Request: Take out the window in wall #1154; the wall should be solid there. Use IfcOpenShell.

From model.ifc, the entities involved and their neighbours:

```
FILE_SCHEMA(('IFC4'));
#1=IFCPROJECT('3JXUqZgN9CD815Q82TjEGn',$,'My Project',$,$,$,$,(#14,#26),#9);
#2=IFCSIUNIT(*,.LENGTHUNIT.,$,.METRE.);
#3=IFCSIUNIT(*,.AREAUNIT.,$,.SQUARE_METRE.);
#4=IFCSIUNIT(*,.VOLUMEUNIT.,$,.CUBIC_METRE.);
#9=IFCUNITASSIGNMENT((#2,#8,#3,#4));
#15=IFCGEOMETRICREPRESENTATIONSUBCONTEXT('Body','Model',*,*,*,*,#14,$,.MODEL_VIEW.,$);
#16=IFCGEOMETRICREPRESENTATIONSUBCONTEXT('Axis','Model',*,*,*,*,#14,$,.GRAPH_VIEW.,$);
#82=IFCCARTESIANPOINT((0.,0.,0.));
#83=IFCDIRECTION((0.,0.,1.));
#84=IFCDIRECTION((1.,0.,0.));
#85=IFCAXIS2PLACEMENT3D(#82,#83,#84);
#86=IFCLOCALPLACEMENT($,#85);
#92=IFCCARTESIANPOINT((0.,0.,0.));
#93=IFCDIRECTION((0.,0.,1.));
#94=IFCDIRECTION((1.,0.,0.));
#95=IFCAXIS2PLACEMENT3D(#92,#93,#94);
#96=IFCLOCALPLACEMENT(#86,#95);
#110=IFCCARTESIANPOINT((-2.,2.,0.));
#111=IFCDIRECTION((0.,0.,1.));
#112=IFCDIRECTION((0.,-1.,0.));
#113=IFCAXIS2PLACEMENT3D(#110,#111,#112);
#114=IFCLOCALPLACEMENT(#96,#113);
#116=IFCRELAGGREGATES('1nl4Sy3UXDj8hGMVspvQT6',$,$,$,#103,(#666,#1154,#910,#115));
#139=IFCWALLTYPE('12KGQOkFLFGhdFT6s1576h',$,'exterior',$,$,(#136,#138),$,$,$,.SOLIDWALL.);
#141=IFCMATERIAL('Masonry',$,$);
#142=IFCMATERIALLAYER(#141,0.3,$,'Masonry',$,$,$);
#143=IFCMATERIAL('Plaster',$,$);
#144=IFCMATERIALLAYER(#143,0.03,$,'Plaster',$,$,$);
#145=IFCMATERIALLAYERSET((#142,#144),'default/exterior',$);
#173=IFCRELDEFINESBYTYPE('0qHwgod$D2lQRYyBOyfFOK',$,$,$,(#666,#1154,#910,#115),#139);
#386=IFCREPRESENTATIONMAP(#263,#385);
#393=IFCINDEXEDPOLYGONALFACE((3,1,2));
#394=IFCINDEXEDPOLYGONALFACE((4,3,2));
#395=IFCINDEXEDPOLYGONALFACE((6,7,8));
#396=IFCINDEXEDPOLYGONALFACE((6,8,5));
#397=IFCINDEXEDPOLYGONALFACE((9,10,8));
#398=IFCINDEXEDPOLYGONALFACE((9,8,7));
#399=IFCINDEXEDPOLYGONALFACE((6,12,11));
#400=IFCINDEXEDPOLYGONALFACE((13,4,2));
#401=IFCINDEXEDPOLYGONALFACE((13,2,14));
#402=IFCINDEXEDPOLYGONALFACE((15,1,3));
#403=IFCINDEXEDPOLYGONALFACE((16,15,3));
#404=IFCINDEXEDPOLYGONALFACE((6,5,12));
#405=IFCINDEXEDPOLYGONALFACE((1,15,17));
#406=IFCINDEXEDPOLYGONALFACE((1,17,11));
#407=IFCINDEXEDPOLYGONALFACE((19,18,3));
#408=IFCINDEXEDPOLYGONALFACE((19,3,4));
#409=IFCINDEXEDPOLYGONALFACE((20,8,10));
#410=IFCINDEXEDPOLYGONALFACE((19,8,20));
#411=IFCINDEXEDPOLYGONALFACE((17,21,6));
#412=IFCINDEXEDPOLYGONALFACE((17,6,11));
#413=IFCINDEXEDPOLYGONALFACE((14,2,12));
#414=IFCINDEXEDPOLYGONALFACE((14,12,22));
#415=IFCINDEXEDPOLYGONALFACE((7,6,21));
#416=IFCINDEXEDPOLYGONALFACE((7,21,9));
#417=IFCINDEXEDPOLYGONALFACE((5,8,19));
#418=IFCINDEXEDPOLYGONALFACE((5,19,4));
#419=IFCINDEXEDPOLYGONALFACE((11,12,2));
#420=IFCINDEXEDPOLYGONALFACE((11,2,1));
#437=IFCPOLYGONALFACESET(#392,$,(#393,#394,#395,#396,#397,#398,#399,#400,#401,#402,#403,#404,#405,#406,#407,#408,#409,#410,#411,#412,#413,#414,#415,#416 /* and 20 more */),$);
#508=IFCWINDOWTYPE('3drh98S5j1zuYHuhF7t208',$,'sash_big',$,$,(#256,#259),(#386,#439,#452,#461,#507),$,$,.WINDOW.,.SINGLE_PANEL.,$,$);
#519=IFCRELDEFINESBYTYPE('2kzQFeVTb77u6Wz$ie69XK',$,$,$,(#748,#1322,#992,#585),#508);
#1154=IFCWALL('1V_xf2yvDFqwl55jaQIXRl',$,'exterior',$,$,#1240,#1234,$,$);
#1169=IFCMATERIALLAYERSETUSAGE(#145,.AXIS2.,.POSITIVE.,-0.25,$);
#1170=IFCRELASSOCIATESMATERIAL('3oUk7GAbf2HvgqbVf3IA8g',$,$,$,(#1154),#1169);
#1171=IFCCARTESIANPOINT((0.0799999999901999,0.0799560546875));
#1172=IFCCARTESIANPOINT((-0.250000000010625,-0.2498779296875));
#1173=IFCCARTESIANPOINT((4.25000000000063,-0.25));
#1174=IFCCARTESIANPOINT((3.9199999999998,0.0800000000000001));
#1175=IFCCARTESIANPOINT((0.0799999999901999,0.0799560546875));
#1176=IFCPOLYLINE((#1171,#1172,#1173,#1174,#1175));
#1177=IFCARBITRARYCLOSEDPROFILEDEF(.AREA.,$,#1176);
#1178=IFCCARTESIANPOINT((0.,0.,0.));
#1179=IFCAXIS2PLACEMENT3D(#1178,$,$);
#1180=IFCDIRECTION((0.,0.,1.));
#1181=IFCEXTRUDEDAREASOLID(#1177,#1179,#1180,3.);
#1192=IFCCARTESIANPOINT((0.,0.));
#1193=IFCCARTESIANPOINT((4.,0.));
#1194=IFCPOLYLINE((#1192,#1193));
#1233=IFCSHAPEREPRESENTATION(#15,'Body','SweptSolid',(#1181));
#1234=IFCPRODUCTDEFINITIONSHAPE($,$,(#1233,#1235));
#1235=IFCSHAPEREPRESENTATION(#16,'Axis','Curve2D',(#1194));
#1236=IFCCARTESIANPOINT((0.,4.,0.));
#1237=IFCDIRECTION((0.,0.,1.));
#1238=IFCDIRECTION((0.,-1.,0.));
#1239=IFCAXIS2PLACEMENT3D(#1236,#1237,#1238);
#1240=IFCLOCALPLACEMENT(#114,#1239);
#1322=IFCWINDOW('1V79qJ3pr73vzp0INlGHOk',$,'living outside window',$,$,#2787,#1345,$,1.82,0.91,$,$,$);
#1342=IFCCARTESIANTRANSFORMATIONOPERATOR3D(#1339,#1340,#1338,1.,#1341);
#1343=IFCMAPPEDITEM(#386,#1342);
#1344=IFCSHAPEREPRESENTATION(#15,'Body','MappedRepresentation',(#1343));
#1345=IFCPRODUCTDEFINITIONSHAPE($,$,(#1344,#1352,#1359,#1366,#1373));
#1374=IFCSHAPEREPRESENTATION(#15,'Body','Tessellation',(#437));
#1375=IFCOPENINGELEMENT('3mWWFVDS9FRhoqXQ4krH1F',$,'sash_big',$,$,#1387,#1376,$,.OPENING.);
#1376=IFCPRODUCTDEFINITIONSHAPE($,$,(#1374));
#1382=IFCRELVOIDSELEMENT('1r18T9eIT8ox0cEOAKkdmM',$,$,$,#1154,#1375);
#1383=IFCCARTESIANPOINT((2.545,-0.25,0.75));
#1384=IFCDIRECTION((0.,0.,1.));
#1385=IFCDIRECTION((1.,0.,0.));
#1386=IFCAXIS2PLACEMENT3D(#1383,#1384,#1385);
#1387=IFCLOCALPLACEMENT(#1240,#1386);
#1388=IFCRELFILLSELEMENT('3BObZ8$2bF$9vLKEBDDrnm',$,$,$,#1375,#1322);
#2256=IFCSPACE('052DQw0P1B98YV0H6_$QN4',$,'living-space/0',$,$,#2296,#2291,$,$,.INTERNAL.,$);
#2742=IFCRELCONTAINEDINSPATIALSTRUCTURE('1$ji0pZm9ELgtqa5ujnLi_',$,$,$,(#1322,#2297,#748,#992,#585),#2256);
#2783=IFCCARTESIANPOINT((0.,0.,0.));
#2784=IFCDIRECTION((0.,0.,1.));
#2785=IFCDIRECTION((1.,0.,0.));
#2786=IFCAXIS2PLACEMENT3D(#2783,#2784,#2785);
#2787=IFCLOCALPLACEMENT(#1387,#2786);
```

```python
import ifcopenshell
import ifcopenshell.api.feature
import ifcopenshell.api.root
import ifcopenshell.geom
import ifcopenshell.util.shape

model = ifcopenshell.open("model.ifc")
settings = ifcopenshell.geom.settings()


def volume(element):
    """Net volume in cubic metres, openings subtracted."""
    shape = ifcopenshell.geom.create_shape(settings, element)
    return ifcopenshell.util.shape.get_volume(shape.geometry)


window = model.by_guid("1V79qJ3pr73vzp0INlGHOk")
opening = window.FillsVoids[0].RelatingOpeningElement
wall = opening.VoidsElements[0].RelatingBuildingElement
before = volume(wall)

ifcopenshell.api.root.remove_product(model, product=window)
ifcopenshell.api.feature.remove_feature(model, feature=opening)

after = volume(wall)

print(f"wall volume {before:.3f} -> {after:.3f} m3")

model.write("model-out.ifc")
```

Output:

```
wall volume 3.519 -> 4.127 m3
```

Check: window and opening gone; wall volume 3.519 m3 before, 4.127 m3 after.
